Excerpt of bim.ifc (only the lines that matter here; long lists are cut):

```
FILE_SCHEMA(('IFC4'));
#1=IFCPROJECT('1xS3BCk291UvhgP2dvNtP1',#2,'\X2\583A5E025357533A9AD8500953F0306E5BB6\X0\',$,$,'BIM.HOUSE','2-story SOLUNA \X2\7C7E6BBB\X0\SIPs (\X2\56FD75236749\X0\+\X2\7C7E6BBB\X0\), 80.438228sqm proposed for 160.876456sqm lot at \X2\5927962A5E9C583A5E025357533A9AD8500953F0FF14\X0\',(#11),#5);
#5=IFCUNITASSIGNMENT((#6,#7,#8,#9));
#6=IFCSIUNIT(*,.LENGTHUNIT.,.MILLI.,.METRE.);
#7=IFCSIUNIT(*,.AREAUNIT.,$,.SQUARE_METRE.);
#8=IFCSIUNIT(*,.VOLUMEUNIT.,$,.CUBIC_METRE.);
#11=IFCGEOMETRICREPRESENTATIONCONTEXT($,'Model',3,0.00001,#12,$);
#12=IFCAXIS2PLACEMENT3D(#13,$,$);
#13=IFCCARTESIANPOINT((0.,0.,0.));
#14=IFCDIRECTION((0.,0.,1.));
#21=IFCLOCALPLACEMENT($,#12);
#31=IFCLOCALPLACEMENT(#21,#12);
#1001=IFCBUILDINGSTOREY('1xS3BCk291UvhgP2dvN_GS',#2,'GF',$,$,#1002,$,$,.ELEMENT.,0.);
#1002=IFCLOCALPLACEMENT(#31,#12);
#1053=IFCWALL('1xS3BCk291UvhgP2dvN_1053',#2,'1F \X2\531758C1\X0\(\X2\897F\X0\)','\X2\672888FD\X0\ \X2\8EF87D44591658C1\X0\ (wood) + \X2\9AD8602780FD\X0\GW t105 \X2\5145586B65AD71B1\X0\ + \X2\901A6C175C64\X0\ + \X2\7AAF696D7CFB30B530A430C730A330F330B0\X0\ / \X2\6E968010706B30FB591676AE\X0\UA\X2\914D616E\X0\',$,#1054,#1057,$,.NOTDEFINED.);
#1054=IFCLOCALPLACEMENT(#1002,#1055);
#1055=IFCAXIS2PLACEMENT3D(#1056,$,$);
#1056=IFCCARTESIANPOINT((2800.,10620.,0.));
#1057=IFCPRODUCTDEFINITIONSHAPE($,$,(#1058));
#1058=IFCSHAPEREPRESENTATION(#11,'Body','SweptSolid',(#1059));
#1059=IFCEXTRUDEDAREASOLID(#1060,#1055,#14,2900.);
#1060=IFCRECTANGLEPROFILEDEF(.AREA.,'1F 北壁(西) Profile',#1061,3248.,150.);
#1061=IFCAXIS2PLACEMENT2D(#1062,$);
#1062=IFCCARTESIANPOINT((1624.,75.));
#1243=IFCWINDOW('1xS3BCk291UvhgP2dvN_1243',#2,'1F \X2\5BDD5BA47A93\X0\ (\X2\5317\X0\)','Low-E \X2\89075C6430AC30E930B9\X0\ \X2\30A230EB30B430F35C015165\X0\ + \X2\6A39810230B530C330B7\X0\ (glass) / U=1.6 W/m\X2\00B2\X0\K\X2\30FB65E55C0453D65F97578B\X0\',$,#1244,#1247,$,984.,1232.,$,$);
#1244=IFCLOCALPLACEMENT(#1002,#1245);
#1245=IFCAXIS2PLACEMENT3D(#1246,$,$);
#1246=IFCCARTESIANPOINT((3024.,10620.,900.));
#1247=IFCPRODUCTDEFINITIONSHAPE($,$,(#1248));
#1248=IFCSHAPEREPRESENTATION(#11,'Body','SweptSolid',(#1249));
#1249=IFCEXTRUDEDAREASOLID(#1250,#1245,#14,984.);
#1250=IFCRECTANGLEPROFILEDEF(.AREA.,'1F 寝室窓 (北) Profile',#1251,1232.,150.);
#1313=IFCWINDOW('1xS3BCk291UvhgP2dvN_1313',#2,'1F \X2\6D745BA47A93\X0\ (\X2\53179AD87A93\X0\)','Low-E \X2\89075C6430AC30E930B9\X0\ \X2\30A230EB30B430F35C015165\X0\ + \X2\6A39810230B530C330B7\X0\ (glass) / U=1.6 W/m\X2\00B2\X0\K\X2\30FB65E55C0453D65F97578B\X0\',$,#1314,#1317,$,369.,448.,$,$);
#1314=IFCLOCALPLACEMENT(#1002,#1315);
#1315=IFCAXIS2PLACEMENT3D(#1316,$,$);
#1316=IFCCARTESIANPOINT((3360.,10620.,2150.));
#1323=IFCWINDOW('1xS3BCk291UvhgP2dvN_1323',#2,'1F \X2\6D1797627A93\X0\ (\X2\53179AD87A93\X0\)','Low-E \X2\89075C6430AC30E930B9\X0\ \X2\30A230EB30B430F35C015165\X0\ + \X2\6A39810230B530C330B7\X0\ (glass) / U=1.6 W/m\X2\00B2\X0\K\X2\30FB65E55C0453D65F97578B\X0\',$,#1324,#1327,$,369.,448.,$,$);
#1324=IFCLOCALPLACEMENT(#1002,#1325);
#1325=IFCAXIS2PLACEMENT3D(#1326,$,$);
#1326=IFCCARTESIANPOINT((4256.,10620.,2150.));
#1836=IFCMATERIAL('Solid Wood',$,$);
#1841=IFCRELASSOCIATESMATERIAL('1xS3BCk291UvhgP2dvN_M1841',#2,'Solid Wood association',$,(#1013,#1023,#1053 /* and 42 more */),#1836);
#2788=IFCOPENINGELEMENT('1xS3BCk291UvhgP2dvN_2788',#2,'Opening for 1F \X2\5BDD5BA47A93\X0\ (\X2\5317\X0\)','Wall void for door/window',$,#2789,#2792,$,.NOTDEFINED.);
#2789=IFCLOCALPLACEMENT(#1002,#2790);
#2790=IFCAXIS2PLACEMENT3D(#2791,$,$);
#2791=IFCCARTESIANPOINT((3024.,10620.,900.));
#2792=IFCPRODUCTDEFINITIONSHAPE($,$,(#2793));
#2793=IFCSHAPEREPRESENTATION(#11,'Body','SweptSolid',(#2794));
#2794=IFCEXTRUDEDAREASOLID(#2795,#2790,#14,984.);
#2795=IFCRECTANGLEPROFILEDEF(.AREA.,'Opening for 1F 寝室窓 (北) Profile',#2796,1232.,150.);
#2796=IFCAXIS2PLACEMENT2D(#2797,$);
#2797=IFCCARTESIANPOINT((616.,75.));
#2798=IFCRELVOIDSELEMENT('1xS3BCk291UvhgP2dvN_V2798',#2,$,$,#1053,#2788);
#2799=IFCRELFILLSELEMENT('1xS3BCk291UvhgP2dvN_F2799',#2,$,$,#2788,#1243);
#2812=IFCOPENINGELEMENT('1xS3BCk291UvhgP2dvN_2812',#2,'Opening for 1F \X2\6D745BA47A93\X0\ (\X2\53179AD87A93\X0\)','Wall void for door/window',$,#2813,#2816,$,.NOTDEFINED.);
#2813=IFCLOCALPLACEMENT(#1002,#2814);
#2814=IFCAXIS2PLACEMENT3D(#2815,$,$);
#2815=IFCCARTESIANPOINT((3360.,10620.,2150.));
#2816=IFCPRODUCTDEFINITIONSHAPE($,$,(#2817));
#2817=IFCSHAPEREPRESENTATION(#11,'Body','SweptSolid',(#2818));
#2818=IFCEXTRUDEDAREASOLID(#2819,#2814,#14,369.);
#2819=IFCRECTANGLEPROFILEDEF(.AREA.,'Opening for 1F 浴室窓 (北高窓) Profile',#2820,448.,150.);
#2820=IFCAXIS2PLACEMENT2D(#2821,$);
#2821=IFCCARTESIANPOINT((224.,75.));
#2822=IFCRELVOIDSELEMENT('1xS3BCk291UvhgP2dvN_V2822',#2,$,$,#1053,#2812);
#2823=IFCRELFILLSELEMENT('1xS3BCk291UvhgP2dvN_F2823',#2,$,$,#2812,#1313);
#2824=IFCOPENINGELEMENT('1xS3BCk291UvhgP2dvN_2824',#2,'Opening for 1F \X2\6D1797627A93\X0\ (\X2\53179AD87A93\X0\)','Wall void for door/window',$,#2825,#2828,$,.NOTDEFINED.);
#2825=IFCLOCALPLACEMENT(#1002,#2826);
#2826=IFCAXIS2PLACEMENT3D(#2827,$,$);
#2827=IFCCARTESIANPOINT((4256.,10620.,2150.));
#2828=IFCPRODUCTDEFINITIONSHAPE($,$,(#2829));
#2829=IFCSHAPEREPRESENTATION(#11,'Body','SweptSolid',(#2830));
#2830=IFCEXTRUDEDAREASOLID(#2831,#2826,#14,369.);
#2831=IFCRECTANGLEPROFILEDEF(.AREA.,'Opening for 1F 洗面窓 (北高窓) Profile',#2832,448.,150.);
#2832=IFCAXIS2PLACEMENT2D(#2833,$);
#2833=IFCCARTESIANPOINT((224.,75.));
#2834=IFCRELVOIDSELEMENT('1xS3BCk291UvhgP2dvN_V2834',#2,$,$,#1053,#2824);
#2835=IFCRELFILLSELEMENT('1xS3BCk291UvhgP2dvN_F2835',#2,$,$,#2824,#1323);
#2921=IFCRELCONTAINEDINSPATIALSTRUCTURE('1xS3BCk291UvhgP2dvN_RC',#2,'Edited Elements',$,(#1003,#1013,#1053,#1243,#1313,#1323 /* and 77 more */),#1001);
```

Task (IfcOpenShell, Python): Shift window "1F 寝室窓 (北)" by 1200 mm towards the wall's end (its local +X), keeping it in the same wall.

```python
import ifcopenshell
import ifcopenshell.api.geometry
import ifcopenshell.util.placement
import ifcopenshell.util.unit

model = ifcopenshell.open("bim.ifc")
unit_scale = ifcopenshell.util.unit.calculate_unit_scale(model)

window = model.by_id(1243)
opening = window.FillsVoids[0].RelatingOpeningElement
wall = opening.VoidsElements[0].RelatingBuildingElement

wall_matrix = ifcopenshell.util.placement.get_local_placement(wall.ObjectPlacement)
shift = wall_matrix[:3, 0] * 1.2 / unit_scale
before = ifcopenshell.util.placement.get_local_placement(window.ObjectPlacement)[:3, 3].copy()

# The window is not placed relative to its opening, so move both.
for product in (opening, window):
    matrix = ifcopenshell.util.placement.get_local_placement(product.ObjectPlacement)
    matrix[:3, 3] += shift
    ifcopenshell.api.geometry.edit_object_placement(model, product=product, matrix=matrix, is_si=False)

after = ifcopenshell.util.placement.get_local_placement(window.ObjectPlacement)[:3, 3]
print("window moved by", (after - before).round(3) + 0.0)

model.write("bim-out.ifc")
```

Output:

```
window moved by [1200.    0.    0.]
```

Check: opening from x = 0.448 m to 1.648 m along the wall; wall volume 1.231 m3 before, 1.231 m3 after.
